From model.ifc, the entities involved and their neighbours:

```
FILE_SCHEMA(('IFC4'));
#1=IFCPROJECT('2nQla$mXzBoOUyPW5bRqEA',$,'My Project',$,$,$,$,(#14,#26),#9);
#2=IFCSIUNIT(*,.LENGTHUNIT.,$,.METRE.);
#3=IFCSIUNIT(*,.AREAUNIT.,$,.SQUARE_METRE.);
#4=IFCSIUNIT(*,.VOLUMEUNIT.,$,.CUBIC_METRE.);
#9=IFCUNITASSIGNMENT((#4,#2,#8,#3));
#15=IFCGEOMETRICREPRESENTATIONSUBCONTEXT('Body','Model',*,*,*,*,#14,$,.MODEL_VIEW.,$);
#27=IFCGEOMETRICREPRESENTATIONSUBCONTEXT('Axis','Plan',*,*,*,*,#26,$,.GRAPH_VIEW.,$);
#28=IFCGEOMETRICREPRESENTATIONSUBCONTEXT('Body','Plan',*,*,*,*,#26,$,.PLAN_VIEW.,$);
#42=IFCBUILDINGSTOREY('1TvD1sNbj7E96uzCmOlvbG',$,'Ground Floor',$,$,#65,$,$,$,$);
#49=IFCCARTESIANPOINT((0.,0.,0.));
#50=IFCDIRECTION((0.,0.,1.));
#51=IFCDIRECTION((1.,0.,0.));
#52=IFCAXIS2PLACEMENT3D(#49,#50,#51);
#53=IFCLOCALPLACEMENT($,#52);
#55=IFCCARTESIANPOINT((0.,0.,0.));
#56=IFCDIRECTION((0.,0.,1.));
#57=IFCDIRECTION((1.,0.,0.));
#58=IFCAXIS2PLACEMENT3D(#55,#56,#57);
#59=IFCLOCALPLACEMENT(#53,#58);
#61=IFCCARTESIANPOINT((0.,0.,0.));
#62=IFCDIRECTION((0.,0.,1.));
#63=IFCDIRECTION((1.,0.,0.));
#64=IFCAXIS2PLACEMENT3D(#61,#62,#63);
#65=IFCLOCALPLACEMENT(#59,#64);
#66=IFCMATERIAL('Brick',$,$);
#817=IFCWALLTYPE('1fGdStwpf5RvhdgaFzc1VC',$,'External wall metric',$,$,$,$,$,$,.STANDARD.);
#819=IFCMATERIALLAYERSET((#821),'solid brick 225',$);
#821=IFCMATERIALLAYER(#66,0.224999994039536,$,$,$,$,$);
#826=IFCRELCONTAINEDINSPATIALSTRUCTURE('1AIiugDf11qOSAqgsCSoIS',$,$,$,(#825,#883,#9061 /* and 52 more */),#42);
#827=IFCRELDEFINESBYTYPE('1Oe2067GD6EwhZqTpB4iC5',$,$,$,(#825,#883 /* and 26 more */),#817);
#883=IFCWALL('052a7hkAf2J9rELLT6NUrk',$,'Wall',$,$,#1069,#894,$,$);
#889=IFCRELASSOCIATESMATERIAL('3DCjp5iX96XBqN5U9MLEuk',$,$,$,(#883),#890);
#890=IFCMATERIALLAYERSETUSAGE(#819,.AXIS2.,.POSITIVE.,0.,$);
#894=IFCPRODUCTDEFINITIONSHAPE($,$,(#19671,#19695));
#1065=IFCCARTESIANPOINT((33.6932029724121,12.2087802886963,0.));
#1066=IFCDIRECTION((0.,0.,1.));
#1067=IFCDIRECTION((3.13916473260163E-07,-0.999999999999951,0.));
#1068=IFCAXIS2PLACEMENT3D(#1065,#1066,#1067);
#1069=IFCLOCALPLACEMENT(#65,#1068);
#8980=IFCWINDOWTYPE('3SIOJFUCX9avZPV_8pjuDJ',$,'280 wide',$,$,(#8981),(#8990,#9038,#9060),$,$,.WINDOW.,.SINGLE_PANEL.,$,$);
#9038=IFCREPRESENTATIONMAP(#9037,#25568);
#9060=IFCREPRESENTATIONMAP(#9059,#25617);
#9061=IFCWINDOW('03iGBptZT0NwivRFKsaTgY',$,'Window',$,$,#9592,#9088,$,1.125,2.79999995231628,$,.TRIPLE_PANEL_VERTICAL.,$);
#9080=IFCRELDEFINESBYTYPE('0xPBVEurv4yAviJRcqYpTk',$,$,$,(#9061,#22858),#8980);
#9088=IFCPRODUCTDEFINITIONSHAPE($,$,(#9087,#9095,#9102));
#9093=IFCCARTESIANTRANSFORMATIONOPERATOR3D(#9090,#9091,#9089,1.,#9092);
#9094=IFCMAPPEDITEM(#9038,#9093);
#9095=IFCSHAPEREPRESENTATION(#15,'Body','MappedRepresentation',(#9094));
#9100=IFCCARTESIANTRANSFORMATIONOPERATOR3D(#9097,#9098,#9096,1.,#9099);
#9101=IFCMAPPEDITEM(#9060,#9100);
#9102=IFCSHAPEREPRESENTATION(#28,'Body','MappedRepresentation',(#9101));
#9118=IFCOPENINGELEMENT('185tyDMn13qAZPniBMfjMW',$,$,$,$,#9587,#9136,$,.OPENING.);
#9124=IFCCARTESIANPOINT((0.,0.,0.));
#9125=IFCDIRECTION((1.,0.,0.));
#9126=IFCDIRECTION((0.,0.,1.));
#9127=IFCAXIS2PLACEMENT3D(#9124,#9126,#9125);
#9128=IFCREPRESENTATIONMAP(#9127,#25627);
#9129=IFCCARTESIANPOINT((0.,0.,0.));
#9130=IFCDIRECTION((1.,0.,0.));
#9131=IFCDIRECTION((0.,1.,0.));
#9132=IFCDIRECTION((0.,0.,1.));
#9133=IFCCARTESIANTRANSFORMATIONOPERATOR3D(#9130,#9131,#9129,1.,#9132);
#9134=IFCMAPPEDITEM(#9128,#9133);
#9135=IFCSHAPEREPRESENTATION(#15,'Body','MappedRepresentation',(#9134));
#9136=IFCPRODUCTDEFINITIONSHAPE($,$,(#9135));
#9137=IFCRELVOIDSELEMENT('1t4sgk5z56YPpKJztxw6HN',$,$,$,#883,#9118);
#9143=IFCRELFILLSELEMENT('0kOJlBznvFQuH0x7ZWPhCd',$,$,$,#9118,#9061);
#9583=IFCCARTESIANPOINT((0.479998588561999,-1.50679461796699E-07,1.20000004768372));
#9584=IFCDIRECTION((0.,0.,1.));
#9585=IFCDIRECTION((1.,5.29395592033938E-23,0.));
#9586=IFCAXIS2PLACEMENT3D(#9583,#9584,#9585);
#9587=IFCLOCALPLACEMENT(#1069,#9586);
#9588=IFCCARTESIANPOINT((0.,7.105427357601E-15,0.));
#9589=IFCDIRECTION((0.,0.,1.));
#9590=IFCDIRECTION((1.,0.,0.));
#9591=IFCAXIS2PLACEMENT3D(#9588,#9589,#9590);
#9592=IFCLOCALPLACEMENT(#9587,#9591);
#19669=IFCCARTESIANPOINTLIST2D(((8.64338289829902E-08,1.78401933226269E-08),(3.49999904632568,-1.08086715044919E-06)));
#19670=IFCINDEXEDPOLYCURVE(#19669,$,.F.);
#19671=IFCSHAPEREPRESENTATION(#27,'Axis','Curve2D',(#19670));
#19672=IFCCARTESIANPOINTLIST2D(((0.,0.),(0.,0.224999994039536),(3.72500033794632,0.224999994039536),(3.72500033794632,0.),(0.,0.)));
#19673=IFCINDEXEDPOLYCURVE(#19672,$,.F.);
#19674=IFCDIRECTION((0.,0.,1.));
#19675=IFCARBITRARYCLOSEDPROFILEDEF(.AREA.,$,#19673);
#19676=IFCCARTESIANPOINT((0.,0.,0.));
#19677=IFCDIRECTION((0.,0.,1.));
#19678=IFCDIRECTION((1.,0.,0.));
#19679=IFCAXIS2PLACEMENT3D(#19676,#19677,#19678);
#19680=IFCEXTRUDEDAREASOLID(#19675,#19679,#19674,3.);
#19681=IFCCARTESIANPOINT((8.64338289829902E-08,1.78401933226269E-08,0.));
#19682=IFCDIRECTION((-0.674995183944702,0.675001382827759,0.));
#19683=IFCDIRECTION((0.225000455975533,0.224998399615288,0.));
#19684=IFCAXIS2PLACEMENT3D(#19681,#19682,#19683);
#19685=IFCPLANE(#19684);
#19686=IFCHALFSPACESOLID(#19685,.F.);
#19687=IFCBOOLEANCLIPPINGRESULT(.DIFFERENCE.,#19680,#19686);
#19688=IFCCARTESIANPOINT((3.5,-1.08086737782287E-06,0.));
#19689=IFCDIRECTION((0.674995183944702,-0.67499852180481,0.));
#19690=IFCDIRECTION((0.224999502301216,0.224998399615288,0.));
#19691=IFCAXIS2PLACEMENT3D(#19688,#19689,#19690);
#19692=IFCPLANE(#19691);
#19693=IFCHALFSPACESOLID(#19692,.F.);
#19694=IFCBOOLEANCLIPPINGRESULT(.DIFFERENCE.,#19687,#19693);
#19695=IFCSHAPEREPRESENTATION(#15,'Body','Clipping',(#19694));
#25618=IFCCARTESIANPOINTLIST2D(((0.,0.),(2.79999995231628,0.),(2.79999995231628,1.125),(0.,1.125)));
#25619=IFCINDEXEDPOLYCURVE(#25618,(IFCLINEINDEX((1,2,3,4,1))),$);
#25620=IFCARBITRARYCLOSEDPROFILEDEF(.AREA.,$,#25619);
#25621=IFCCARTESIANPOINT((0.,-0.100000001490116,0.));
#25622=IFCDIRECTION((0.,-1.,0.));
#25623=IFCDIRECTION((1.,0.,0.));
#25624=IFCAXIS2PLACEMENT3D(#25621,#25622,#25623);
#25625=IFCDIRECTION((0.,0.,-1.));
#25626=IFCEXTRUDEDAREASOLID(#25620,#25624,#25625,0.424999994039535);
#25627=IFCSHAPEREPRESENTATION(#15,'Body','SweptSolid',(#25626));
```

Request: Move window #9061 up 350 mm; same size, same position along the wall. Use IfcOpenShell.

```python
import numpy as np
import ifcopenshell
import ifcopenshell.api.geometry
import ifcopenshell.util.placement
import ifcopenshell.util.unit

model = ifcopenshell.open("model.ifc")
unit_scale = ifcopenshell.util.unit.calculate_unit_scale(model)

window = model.by_guid("03iGBptZT0NwivRFKsaTgY")
opening = window.FillsVoids[0].RelatingOpeningElement
dz = 0.35 / unit_scale

shift = np.array([0.0, 0.0, dz])
# The window is placed relative to its opening, so it follows when the opening moves.
matrix = ifcopenshell.util.placement.get_local_placement(opening.ObjectPlacement)
matrix[:3, 3] += shift
ifcopenshell.api.geometry.edit_object_placement(
    model, product=opening, matrix=matrix, is_si=False, should_transform_children=True
)

print(f"moved by {dz * unit_scale:+.3f} m")

model.write("model_rev.ifc")
```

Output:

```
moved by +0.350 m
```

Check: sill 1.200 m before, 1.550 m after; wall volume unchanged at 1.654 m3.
